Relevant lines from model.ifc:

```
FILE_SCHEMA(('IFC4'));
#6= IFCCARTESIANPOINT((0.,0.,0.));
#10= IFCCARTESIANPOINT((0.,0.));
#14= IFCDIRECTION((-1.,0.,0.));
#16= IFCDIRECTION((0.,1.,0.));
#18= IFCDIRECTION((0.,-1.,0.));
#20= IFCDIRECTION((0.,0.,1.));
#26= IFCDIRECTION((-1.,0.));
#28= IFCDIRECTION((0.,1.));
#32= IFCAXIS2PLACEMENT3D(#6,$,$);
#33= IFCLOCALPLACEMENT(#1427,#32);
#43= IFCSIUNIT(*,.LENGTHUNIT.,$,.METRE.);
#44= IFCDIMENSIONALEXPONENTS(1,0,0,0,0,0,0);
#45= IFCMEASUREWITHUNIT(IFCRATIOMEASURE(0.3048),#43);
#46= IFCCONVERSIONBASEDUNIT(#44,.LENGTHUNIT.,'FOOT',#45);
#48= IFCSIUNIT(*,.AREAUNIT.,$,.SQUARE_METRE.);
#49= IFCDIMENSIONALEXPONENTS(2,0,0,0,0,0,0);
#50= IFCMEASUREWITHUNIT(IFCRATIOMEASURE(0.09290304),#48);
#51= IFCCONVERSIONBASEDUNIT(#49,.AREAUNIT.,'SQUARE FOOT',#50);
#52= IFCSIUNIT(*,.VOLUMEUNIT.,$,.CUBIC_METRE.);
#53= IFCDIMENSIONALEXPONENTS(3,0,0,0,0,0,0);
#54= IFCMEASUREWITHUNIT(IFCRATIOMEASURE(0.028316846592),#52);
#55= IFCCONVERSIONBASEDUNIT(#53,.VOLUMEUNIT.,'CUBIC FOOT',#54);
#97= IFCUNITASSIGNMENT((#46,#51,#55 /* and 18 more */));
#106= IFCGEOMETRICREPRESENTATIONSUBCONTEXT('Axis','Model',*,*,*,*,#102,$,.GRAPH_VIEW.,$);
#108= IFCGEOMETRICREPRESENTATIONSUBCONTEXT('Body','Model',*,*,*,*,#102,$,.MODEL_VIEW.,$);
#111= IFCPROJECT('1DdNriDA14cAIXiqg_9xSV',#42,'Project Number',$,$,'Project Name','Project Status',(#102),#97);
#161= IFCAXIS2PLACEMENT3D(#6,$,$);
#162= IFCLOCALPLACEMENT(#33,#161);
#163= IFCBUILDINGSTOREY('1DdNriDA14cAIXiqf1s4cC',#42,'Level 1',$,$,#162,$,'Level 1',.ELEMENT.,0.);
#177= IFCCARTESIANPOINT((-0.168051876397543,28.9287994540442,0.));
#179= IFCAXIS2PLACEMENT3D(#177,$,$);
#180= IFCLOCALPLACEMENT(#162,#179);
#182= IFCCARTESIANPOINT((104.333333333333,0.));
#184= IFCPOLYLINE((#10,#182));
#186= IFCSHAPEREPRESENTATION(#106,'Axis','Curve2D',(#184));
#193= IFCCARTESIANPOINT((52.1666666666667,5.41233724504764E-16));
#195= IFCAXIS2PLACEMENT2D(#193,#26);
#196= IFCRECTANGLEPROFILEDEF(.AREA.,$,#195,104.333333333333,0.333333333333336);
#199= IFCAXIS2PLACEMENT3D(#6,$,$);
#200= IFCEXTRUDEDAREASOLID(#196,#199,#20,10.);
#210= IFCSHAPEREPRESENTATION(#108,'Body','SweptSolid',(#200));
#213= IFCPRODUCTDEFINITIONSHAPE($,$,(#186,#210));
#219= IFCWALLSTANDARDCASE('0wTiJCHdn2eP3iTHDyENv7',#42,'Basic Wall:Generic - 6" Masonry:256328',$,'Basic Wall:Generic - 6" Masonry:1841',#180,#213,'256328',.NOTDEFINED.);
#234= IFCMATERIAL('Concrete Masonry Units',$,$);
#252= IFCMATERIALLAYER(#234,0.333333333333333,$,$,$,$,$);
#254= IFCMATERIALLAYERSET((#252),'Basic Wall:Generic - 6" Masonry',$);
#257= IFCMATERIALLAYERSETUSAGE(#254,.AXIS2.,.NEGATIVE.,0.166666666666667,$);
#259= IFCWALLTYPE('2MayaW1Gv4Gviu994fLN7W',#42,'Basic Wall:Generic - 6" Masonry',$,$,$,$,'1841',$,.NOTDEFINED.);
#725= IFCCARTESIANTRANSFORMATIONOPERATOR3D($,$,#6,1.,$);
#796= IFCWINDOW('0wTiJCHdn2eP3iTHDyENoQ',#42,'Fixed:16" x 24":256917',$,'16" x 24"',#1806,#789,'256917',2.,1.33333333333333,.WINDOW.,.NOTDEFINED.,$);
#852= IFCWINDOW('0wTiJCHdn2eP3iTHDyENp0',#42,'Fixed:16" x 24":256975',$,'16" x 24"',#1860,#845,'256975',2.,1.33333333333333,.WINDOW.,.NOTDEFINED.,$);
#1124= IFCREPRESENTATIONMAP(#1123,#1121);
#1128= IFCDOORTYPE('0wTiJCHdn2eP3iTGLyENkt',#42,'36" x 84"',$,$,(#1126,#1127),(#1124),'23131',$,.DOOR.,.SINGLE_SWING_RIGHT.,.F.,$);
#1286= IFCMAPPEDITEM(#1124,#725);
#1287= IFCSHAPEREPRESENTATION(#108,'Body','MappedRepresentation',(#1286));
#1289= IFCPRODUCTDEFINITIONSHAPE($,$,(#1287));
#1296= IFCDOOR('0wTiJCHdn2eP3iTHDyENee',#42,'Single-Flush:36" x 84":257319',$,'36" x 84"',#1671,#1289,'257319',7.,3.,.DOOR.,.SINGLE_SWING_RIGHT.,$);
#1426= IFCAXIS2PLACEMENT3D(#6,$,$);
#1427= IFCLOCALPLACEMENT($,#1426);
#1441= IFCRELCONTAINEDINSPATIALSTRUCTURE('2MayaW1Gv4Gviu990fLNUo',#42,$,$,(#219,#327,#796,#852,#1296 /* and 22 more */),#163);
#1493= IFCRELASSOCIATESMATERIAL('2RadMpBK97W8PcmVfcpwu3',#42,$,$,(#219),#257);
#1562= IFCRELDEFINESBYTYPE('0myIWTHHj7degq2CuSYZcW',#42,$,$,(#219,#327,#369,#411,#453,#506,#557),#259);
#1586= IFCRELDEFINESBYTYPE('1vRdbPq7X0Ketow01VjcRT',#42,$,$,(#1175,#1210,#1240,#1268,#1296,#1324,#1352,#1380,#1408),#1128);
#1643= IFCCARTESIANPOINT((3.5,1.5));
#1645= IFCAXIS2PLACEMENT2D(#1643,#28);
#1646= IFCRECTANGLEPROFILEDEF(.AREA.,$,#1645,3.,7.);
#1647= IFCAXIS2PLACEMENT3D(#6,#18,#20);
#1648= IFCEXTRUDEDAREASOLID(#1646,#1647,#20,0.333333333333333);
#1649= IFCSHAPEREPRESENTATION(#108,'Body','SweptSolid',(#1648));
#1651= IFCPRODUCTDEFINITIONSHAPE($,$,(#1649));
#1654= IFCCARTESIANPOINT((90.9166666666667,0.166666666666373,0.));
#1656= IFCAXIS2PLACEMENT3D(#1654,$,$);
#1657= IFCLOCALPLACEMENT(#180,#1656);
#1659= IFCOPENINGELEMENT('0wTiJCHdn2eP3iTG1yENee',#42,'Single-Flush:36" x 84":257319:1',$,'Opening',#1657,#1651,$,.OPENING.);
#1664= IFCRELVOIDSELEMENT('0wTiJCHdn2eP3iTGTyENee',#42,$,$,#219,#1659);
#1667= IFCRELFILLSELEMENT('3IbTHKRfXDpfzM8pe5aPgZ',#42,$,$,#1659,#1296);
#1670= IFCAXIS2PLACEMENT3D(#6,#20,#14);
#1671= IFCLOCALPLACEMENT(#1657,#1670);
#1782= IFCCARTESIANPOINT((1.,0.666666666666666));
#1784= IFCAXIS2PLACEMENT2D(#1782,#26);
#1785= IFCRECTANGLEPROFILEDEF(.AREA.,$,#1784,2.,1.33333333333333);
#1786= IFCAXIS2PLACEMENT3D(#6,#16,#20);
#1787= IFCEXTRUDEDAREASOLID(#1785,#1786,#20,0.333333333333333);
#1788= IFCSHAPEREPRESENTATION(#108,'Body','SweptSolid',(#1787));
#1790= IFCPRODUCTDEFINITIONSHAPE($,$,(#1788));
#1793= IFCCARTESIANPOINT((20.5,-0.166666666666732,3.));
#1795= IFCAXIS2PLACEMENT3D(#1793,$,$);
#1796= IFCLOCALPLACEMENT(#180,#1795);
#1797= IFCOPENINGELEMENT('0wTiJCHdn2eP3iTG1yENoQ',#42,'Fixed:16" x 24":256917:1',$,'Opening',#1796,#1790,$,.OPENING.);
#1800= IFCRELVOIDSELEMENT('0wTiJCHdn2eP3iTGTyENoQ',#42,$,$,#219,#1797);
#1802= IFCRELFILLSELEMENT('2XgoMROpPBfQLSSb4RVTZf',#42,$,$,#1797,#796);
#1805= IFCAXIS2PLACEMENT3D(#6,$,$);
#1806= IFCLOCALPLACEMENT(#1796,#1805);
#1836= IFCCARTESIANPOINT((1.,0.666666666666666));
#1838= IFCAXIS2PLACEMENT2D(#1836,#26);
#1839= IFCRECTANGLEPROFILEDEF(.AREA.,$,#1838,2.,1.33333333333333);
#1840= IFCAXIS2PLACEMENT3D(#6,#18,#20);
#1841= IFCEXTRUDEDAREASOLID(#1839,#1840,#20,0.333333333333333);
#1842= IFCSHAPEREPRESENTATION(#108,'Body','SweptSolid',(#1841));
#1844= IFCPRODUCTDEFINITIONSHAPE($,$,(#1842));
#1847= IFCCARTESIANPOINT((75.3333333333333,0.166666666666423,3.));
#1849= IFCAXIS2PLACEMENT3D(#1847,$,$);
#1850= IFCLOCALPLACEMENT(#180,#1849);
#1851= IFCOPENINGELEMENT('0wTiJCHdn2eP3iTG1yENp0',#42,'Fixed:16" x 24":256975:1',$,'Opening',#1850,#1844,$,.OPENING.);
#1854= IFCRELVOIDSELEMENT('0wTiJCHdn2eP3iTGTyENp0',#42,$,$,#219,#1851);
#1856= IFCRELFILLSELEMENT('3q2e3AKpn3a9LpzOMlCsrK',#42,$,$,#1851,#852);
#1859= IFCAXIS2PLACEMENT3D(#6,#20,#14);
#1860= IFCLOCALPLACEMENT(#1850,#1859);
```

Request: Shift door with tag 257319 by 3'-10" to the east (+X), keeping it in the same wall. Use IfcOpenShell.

```python
import ifcopenshell
import ifcopenshell.api.geometry
import ifcopenshell.util.placement
import ifcopenshell.util.unit

model = ifcopenshell.open("model.ifc")
unit_scale = ifcopenshell.util.unit.calculate_unit_scale(model)

door = model.by_guid("0wTiJCHdn2eP3iTHDyENee")
opening = door.FillsVoids[0].RelatingOpeningElement
wall = opening.VoidsElements[0].RelatingBuildingElement

wall_matrix = ifcopenshell.util.placement.get_local_placement(wall.ObjectPlacement)
shift = wall_matrix[:3, 0] * 46 * 0.0254 / unit_scale
before = ifcopenshell.util.placement.get_local_placement(door.ObjectPlacement)[:3, 3].copy()

# The door is placed relative to its opening, so it follows when the opening moves.
matrix = ifcopenshell.util.placement.get_local_placement(opening.ObjectPlacement)
matrix[:3, 3] += shift
ifcopenshell.api.geometry.edit_object_placement(
    model, product=opening, matrix=matrix, is_si=False, should_transform_children=True
)

after = ifcopenshell.util.placement.get_local_placement(door.ObjectPlacement)[:3, 3]
print("door moved by", (after - before).round(3) + 0.0)

model.write("model_updated.ifc")
```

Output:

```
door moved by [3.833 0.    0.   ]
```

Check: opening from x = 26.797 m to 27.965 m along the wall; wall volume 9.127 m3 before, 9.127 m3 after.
